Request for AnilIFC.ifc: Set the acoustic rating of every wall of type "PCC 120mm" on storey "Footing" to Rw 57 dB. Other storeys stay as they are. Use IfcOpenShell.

First a look at what the model holds.

```python
import ifcopenshell
import ifcopenshell.util.element

model = ifcopenshell.open("AnilIFC.ifc")
print(model.schema)
storey = next(s for s in model.by_type("IfcBuildingStorey") if s.Name == "Footing")
walls = [e for e in ifcopenshell.util.element.get_decomposition(storey) if e.is_a("IfcWall")]
seen = {}
for e in walls:
    element_type = ifcopenshell.util.element.get_type(e)
    key = (element_type.Name if element_type != e and element_type else None, ifcopenshell.util.element.get_pset(e, "Pset_WallCommon", "AcousticRating"))
    seen[key] = seen.get(key, 0) + 1
for (name, value), count in sorted(seen.items(), key=str):
    print(count, "x", name, "|", value)
```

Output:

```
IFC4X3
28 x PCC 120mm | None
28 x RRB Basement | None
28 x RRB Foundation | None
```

```python
import ifcopenshell
import ifcopenshell.api.pset
import ifcopenshell.util.element

model = ifcopenshell.open("AnilIFC.ifc")

storey = next(s for s in model.by_type("IfcBuildingStorey") if s.Name == "Footing")
walls = [e for e in ifcopenshell.util.element.get_decomposition(storey) if e.is_a("IfcWall")]

count = 0
for e in walls:
    element_type = ifcopenshell.util.element.get_type(e)
    if element_type in (None, e) or element_type.Name != "PCC 120mm":
        continue
    # add_pset returns the element's existing set when there is one.
    pset = ifcopenshell.api.pset.add_pset(model, product=e, name="Pset_WallCommon")
    ifcopenshell.api.pset.edit_pset(model, pset=pset, properties={"AcousticRating": "Rw 57 dB"})
    count += 1

print(count, "walls updated")

model.write("AnilIFC_edited.ifc")
```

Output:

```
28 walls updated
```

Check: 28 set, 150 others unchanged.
